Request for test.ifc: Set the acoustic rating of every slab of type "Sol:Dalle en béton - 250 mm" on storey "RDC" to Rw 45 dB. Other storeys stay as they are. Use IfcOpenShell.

First a look at what the model holds.

```python
import ifcopenshell
import ifcopenshell.util.element

model = ifcopenshell.open("test.ifc")
print(model.schema)
storey = next(s for s in model.by_type("IfcBuildingStorey") if s.Name == "RDC")
slabs = [e for e in ifcopenshell.util.element.get_decomposition(storey) if e.is_a("IfcSlab")]
seen = {}
for e in slabs:
    element_type = ifcopenshell.util.element.get_type(e)
    key = (element_type.Name if element_type != e and element_type else None, ifcopenshell.util.element.get_pset(e, "Pset_SlabCommon", "AcousticRating"))
    seen[key] = seen.get(key, 0) + 1
for (name, value), count in sorted(seen.items(), key=str):
    print(count, "x", name, "|", value)
```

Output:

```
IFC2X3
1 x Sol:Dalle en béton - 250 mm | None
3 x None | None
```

```python
import ifcopenshell
import ifcopenshell.api.pset
import ifcopenshell.util.element

model = ifcopenshell.open("test.ifc")

storey = next(s for s in model.by_type("IfcBuildingStorey") if s.Name == "RDC")
slabs = [e for e in ifcopenshell.util.element.get_decomposition(storey) if e.is_a("IfcSlab")]

count = 0
for e in slabs:
    element_type = ifcopenshell.util.element.get_type(e)
    if element_type in (None, e) or element_type.Name != "Sol:Dalle en béton - 250 mm":
        continue
    # add_pset returns the element's existing set when there is one.
    pset = ifcopenshell.api.pset.add_pset(model, product=e, name="Pset_SlabCommon")
    ifcopenshell.api.pset.edit_pset(model, pset=pset, properties={"AcousticRating": "Rw 45 dB"})
    count += 1

print(count, "slabs updated")

model.write("test_updated.ifc")
```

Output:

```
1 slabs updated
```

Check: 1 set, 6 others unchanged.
